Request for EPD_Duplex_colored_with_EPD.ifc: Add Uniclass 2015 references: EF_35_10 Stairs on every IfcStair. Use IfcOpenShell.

First a look at what the model holds.

```python
import ifcopenshell

model = ifcopenshell.open("EPD_Duplex_colored_with_EPD.ifc")
print(model.schema)
print("classifications:", [c.Name for c in model.by_type("IfcClassification")])
for ifc_class in ("IfcDoor", "IfcRoof", "IfcStair", "IfcWall", "IfcWindow"):
    print(ifc_class, len(model.by_type(ifc_class)))
```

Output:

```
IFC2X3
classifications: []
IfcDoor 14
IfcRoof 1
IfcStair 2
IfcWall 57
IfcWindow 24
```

```python
import ifcopenshell
import ifcopenshell.api.classification

model = ifcopenshell.open("EPD_Duplex_colored_with_EPD.ifc")

# IFC2X3 requires Source and Edition and has no link from the project to the system.
system = model.create_entity("IfcClassification", Source="NBS", Edition="2015", Name="Uniclass 2015")

codes = {
    "IfcStair": ("EF_35_10", "Stairs"),
}
for ifc_class, (code, name) in codes.items():
    products = model.by_type(ifc_class)
    ifcopenshell.api.classification.add_reference(
        model, products=products, classification=system, identification=code, name=name
    )
    print(code, len(products))

model.write("EPD_Duplex_colored_with_EPD_updated.ifc")
```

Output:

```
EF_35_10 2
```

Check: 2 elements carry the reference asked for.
